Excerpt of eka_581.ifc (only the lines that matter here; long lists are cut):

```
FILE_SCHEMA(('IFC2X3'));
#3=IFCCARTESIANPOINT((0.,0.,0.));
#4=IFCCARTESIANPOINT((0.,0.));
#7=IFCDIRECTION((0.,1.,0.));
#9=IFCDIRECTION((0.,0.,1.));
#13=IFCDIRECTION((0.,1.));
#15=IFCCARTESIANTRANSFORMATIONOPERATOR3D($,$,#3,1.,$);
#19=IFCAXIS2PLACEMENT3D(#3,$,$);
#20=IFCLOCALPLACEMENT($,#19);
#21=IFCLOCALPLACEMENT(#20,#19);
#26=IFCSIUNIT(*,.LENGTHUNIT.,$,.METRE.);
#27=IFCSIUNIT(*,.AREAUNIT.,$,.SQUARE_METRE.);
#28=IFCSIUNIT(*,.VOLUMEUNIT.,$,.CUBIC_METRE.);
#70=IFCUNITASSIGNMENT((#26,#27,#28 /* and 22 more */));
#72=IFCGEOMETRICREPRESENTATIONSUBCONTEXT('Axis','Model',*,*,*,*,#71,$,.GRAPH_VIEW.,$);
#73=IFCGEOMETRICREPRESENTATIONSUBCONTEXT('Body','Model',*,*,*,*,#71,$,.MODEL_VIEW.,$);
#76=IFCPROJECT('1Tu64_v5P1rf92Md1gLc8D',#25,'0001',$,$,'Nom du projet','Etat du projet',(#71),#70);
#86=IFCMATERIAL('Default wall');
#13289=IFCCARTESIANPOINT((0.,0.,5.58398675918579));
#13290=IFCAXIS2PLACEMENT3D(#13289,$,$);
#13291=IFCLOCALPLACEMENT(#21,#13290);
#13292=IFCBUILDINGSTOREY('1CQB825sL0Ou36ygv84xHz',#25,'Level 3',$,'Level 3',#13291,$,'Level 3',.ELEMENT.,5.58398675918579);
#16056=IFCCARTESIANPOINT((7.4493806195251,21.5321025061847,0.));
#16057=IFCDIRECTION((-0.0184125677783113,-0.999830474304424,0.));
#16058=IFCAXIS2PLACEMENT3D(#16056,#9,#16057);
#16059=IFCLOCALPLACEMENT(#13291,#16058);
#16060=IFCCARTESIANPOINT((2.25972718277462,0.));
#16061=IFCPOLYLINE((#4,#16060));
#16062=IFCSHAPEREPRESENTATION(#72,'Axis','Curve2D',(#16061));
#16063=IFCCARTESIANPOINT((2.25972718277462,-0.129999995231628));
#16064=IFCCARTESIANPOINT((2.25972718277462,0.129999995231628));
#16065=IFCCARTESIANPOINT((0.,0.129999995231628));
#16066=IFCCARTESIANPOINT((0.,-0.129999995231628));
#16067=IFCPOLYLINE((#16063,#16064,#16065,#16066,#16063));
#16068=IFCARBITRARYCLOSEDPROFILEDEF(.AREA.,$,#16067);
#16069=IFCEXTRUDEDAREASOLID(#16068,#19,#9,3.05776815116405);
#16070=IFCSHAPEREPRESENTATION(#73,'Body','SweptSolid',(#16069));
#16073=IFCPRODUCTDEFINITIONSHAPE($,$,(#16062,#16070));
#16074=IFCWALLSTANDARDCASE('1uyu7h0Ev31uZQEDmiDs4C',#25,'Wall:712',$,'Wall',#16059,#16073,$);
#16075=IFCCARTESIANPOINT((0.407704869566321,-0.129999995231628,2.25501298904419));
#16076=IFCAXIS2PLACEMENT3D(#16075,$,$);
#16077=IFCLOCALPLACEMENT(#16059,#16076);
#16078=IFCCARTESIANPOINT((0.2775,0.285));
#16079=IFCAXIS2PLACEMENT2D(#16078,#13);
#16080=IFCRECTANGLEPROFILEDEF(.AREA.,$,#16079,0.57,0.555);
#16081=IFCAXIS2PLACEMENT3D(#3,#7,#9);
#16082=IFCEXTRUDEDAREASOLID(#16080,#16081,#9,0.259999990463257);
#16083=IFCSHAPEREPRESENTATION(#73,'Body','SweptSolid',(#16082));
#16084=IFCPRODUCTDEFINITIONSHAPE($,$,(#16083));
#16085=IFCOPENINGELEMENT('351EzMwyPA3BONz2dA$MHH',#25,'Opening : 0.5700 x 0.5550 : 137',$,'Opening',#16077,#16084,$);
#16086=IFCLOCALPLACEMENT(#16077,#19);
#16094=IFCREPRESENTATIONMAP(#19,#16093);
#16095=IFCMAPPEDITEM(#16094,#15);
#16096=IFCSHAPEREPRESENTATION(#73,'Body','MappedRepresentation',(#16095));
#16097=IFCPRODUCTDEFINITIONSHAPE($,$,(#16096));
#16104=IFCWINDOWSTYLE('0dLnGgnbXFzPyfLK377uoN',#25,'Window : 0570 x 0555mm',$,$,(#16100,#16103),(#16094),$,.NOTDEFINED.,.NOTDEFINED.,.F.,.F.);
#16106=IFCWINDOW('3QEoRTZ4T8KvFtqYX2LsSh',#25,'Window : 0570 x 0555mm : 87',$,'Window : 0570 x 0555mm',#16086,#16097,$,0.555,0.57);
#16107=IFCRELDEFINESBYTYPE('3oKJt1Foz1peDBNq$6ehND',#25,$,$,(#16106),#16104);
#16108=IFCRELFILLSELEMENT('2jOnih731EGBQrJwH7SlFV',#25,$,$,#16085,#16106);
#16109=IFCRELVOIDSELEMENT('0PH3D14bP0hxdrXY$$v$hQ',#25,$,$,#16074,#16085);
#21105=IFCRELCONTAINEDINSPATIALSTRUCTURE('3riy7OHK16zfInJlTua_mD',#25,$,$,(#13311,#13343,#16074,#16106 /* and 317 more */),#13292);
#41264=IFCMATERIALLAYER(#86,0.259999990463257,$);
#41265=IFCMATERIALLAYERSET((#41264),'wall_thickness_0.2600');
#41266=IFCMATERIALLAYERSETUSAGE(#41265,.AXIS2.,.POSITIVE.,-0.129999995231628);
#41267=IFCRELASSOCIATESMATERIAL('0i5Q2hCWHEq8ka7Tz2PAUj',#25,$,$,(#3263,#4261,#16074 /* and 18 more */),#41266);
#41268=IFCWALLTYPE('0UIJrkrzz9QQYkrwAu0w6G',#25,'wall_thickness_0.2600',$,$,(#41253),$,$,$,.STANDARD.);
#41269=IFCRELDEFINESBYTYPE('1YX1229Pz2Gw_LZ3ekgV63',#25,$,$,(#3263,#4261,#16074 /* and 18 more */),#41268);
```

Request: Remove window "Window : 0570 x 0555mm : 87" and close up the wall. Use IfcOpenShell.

```python
import ifcopenshell
import ifcopenshell.api.feature
import ifcopenshell.api.root
import ifcopenshell.geom
import ifcopenshell.util.shape

model = ifcopenshell.open("eka_581.ifc")
settings = ifcopenshell.geom.settings()


def volume(element):
    """Net volume in cubic metres, openings subtracted."""
    shape = ifcopenshell.geom.create_shape(settings, element)
    return ifcopenshell.util.shape.get_volume(shape.geometry)


window = model.by_id(16106)
opening = window.FillsVoids[0].RelatingOpeningElement
wall = opening.VoidsElements[0].RelatingBuildingElement
before = volume(wall)

ifcopenshell.api.root.remove_product(model, product=window)
ifcopenshell.api.feature.remove_feature(model, feature=opening)

after = volume(wall)

print(f"wall volume {before:.3f} -> {after:.3f} m3")

model.write("eka_581_updated.ifc")
```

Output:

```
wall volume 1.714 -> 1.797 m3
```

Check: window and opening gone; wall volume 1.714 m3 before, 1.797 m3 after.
